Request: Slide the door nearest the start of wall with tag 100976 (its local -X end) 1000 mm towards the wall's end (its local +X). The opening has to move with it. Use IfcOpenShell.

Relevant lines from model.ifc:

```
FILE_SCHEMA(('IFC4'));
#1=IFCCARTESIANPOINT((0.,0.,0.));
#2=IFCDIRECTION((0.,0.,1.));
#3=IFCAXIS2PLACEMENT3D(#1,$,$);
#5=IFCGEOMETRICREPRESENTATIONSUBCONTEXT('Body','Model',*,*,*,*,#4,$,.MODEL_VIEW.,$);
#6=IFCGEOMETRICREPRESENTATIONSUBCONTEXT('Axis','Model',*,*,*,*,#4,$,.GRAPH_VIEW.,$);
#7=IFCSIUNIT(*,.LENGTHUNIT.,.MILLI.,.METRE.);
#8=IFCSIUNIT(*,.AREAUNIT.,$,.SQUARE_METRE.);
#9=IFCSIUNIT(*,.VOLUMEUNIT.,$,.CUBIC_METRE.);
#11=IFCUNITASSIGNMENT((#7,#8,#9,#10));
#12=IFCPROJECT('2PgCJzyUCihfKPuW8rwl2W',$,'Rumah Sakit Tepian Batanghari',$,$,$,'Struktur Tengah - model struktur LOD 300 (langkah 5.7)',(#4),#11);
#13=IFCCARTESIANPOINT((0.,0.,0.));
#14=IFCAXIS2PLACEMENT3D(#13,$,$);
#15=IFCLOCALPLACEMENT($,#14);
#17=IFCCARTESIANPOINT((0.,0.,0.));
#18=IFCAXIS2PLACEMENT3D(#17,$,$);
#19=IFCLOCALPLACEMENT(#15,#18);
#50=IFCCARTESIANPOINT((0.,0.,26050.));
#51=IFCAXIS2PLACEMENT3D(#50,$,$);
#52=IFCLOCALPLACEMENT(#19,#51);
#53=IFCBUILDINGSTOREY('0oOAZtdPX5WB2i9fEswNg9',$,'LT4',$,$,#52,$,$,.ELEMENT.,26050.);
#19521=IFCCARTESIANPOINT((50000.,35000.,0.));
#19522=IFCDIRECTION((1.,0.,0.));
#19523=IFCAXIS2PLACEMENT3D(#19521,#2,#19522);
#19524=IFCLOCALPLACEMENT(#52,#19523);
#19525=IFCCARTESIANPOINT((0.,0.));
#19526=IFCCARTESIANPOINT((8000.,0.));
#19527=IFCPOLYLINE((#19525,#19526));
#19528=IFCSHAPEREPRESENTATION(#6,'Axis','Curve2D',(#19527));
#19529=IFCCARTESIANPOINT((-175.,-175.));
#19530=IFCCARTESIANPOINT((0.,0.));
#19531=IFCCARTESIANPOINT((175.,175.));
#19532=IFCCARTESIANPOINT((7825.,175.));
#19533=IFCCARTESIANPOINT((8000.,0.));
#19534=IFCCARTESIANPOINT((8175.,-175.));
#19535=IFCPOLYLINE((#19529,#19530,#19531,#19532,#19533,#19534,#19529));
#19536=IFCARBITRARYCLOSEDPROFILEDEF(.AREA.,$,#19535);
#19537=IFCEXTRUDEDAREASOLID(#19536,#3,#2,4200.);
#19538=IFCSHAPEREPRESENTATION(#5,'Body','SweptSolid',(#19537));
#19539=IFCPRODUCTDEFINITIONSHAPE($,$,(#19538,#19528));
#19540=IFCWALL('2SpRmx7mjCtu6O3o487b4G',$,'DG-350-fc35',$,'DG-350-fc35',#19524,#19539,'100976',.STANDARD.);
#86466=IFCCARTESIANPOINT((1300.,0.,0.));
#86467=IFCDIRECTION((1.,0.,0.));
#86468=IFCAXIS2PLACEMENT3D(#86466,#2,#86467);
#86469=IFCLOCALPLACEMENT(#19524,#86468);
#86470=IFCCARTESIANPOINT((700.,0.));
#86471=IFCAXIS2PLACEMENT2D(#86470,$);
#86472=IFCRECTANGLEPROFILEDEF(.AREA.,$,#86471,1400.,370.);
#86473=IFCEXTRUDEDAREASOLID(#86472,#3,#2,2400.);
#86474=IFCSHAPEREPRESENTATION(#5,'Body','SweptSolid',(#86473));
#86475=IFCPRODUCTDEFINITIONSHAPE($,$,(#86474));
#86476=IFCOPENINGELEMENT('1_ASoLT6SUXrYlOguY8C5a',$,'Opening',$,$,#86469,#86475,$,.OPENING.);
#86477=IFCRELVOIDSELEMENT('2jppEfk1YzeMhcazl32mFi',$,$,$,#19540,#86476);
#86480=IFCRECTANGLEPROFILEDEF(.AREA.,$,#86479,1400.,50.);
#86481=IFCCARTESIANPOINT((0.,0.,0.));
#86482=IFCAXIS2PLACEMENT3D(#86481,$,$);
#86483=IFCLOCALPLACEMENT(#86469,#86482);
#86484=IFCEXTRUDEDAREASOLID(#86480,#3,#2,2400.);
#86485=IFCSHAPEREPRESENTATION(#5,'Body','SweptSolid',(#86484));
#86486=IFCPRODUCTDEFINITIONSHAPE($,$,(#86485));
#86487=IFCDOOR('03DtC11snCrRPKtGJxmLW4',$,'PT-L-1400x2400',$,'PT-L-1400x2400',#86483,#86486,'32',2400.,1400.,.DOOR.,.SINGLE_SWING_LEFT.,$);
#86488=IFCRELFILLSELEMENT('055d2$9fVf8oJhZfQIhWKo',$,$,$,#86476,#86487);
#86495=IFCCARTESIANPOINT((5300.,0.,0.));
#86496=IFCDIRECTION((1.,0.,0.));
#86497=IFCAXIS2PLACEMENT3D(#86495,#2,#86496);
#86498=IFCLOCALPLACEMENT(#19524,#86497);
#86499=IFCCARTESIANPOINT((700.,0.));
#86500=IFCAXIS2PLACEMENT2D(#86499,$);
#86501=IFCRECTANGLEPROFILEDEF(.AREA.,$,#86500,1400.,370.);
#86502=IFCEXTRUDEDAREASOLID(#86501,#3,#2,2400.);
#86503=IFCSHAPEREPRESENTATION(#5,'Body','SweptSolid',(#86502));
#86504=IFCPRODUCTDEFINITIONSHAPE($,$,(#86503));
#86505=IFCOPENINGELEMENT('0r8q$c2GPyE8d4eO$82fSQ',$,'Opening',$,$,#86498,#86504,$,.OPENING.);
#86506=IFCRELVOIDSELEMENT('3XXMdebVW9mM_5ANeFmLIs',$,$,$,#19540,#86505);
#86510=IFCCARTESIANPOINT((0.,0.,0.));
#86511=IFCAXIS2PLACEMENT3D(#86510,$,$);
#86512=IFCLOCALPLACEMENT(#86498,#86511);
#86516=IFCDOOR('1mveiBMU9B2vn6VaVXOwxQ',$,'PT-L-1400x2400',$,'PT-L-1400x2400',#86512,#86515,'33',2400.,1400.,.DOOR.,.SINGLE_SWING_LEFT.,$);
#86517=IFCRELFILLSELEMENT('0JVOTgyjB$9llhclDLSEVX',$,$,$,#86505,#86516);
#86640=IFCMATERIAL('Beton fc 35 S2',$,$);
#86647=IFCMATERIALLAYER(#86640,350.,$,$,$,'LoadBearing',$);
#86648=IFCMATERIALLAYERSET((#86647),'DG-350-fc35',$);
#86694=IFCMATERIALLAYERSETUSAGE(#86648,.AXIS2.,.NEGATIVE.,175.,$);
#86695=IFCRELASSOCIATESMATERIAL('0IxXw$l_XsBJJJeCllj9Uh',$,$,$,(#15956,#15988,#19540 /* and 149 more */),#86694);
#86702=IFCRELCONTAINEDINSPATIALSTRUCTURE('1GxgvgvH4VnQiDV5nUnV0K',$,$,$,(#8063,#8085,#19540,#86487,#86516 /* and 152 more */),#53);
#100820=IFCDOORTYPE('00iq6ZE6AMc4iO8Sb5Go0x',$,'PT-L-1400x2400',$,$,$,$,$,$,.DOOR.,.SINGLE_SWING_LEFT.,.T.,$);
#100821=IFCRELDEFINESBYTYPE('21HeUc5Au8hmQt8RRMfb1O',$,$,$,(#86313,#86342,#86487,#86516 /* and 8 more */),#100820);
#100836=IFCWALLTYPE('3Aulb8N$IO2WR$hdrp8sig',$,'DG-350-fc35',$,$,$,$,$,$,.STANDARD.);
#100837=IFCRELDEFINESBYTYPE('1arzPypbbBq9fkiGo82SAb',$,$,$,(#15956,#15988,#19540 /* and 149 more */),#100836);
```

```python
import ifcopenshell
import ifcopenshell.api.geometry
import ifcopenshell.util.placement

model = ifcopenshell.open("model.ifc")

door = model.by_id(86487)
opening = door.FillsVoids[0].RelatingOpeningElement
wall = opening.VoidsElements[0].RelatingBuildingElement

wall_matrix = ifcopenshell.util.placement.get_local_placement(wall.ObjectPlacement)
shift = wall_matrix[:3, 0] * 1000.0
before = ifcopenshell.util.placement.get_local_placement(door.ObjectPlacement)[:3, 3].copy()

# The door is placed relative to its opening, so it follows when the opening moves.
matrix = ifcopenshell.util.placement.get_local_placement(opening.ObjectPlacement)
matrix[:3, 3] += shift
ifcopenshell.api.geometry.edit_object_placement(
    model, product=opening, matrix=matrix, is_si=False, should_transform_children=True
)

after = ifcopenshell.util.placement.get_local_placement(door.ObjectPlacement)[:3, 3]
print("door moved by", (after - before).round(3) + 0.0)

model.write("model_v2.ifc")
```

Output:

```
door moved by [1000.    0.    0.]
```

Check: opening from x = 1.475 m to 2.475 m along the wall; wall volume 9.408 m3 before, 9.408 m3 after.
